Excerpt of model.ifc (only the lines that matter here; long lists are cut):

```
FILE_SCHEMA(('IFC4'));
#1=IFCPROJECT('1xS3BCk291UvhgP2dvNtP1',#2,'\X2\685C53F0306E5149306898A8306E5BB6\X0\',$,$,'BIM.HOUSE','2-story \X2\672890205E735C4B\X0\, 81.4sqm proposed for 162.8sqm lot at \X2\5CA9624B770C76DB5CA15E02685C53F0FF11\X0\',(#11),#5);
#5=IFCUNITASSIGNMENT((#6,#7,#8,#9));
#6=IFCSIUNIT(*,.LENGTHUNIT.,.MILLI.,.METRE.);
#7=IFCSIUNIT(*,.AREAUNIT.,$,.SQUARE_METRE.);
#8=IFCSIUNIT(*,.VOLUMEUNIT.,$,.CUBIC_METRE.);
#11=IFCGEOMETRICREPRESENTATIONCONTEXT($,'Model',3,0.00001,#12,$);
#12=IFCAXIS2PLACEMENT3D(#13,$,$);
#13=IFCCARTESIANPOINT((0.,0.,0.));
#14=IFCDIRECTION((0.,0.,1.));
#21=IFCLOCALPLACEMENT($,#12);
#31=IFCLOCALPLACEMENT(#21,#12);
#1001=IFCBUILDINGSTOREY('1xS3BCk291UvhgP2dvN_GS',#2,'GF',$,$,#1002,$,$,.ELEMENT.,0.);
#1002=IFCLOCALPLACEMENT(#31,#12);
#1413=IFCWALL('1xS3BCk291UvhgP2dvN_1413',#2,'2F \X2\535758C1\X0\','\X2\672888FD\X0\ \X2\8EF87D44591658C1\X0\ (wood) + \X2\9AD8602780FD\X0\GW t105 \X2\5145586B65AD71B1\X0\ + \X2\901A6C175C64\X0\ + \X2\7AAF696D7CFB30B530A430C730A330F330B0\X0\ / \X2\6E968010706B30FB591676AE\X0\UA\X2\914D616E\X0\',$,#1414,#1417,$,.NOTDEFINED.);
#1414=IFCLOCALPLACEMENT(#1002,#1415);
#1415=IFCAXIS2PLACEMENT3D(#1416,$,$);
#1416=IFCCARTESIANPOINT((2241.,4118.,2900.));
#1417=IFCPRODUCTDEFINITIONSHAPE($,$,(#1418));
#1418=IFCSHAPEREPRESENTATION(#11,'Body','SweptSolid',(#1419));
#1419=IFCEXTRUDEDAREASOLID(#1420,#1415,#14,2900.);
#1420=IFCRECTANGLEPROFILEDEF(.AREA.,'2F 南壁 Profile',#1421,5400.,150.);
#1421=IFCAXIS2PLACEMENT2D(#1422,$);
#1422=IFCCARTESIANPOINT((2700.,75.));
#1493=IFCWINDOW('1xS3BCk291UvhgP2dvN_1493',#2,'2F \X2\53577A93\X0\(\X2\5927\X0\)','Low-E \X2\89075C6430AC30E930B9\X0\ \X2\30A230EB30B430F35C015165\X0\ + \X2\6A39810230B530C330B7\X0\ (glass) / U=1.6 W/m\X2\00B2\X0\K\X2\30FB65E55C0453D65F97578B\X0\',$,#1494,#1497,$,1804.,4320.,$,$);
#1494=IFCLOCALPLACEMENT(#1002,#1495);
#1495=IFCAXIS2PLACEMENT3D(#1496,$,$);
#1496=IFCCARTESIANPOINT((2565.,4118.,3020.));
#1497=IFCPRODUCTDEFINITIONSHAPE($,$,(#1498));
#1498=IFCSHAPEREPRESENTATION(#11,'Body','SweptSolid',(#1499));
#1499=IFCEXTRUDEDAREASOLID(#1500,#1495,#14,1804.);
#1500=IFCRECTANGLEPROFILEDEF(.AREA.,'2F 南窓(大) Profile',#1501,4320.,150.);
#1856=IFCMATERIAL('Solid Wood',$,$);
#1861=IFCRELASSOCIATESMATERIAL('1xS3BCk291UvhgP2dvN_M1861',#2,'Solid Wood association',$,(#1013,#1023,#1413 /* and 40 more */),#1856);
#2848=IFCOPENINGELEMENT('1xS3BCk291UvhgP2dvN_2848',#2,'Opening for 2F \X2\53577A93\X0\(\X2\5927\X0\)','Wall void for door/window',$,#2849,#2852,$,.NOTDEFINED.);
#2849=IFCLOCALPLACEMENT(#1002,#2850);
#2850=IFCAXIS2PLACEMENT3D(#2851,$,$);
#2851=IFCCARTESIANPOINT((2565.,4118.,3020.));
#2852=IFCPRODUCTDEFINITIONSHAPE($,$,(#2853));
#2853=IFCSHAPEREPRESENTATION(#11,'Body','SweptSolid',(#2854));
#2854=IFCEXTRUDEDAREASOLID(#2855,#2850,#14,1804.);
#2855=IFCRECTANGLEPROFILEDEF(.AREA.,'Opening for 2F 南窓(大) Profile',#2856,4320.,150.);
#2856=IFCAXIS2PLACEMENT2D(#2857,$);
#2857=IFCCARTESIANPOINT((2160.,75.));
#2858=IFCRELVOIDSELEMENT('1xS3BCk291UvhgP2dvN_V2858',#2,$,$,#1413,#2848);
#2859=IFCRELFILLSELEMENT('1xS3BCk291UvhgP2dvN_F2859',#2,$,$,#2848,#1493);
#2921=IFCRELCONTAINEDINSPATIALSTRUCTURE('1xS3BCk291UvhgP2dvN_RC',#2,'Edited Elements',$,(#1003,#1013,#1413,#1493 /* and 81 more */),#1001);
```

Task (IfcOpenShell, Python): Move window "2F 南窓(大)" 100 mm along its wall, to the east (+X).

```python
import ifcopenshell
import ifcopenshell.api.geometry
import ifcopenshell.util.placement

model = ifcopenshell.open("model.ifc")

window = model.by_id(1493)
opening = window.FillsVoids[0].RelatingOpeningElement
wall = opening.VoidsElements[0].RelatingBuildingElement

wall_matrix = ifcopenshell.util.placement.get_local_placement(wall.ObjectPlacement)
shift = wall_matrix[:3, 0] * 100.0
before = ifcopenshell.util.placement.get_local_placement(window.ObjectPlacement)[:3, 3].copy()

# The window is not placed relative to its opening, so move both.
for product in (opening, window):
    matrix = ifcopenshell.util.placement.get_local_placement(product.ObjectPlacement)
    matrix[:3, 3] += shift
    ifcopenshell.api.geometry.edit_object_placement(model, product=product, matrix=matrix, is_si=False)

after = ifcopenshell.util.placement.get_local_placement(window.ObjectPlacement)[:3, 3]
print("window moved by", (after - before).round(3) + 0.0)

model.write("model_edited.ifc")
```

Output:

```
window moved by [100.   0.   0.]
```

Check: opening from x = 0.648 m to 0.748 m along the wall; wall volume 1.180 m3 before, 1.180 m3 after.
